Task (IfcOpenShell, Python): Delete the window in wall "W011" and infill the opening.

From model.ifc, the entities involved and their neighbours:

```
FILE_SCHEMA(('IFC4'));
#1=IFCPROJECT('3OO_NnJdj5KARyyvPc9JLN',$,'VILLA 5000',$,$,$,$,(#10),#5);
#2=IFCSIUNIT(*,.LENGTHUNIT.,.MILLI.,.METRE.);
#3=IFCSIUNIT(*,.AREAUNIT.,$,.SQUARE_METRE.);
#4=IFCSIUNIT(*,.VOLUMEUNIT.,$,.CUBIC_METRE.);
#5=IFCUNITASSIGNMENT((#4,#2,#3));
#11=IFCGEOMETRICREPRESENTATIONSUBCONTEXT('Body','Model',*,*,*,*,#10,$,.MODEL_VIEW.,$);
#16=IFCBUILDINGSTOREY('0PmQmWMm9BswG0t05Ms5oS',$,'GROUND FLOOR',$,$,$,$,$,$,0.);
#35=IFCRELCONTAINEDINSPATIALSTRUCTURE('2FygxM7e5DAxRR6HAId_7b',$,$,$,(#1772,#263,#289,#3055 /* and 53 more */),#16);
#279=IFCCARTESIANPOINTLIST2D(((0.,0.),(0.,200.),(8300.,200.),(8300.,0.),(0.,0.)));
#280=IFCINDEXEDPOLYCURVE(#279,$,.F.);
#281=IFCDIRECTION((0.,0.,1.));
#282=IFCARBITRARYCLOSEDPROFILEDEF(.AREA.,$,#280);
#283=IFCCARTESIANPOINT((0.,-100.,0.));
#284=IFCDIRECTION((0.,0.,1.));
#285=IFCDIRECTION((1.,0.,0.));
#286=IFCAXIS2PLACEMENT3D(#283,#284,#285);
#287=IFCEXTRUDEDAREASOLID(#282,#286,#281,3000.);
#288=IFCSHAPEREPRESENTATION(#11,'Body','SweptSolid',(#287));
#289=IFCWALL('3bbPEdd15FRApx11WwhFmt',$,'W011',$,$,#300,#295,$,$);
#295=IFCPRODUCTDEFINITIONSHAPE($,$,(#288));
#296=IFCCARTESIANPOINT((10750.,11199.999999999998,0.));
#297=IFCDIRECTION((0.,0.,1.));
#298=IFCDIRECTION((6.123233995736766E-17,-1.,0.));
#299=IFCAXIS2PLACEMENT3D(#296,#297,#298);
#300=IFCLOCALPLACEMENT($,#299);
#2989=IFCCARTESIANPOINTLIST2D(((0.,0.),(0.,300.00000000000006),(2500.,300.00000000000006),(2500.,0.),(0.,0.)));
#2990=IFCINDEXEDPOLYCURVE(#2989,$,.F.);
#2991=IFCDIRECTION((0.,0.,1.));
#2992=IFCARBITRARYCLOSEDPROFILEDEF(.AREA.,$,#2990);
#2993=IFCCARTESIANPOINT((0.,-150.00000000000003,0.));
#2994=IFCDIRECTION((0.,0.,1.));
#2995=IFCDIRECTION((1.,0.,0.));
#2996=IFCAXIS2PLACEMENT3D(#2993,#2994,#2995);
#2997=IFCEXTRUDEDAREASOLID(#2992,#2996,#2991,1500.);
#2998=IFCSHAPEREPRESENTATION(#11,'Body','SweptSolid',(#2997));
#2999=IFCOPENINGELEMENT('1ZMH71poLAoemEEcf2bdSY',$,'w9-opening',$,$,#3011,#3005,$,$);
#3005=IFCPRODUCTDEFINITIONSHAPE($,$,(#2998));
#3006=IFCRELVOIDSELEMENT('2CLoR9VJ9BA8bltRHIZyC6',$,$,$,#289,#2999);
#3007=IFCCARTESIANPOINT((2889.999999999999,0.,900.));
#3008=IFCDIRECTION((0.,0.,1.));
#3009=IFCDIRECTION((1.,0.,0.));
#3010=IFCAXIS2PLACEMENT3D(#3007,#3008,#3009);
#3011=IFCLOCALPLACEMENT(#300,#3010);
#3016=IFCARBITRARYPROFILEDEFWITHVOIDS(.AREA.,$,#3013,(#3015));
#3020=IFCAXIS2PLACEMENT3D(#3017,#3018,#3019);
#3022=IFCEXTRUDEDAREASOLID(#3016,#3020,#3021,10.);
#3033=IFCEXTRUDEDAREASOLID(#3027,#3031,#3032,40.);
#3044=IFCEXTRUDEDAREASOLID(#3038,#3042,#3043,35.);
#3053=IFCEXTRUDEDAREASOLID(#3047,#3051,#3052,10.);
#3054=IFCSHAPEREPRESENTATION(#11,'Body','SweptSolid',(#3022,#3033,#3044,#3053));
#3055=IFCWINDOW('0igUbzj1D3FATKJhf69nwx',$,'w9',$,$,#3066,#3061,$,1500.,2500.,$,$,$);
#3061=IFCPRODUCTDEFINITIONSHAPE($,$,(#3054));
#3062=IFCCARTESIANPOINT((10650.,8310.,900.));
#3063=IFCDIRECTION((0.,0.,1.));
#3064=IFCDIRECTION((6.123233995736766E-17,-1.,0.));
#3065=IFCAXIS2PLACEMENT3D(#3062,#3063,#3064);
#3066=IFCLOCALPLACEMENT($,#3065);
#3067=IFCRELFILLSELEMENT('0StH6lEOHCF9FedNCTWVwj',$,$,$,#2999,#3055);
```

```python
import ifcopenshell
import ifcopenshell.api.feature
import ifcopenshell.api.root
import ifcopenshell.geom
import ifcopenshell.util.shape

model = ifcopenshell.open("model.ifc")
settings = ifcopenshell.geom.settings()


def volume(element):
    """Net volume in cubic metres, openings subtracted."""
    shape = ifcopenshell.geom.create_shape(settings, element)
    return ifcopenshell.util.shape.get_volume(shape.geometry)


window = model.by_id(3055)
opening = window.FillsVoids[0].RelatingOpeningElement
wall = opening.VoidsElements[0].RelatingBuildingElement
before = volume(wall)

ifcopenshell.api.root.remove_product(model, product=window)
ifcopenshell.api.feature.remove_feature(model, feature=opening)

after = volume(wall)

print(f"wall volume {before:.3f} -> {after:.3f} m3")

model.write("model-out.ifc")
```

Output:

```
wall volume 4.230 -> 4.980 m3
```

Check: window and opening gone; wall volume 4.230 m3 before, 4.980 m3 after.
